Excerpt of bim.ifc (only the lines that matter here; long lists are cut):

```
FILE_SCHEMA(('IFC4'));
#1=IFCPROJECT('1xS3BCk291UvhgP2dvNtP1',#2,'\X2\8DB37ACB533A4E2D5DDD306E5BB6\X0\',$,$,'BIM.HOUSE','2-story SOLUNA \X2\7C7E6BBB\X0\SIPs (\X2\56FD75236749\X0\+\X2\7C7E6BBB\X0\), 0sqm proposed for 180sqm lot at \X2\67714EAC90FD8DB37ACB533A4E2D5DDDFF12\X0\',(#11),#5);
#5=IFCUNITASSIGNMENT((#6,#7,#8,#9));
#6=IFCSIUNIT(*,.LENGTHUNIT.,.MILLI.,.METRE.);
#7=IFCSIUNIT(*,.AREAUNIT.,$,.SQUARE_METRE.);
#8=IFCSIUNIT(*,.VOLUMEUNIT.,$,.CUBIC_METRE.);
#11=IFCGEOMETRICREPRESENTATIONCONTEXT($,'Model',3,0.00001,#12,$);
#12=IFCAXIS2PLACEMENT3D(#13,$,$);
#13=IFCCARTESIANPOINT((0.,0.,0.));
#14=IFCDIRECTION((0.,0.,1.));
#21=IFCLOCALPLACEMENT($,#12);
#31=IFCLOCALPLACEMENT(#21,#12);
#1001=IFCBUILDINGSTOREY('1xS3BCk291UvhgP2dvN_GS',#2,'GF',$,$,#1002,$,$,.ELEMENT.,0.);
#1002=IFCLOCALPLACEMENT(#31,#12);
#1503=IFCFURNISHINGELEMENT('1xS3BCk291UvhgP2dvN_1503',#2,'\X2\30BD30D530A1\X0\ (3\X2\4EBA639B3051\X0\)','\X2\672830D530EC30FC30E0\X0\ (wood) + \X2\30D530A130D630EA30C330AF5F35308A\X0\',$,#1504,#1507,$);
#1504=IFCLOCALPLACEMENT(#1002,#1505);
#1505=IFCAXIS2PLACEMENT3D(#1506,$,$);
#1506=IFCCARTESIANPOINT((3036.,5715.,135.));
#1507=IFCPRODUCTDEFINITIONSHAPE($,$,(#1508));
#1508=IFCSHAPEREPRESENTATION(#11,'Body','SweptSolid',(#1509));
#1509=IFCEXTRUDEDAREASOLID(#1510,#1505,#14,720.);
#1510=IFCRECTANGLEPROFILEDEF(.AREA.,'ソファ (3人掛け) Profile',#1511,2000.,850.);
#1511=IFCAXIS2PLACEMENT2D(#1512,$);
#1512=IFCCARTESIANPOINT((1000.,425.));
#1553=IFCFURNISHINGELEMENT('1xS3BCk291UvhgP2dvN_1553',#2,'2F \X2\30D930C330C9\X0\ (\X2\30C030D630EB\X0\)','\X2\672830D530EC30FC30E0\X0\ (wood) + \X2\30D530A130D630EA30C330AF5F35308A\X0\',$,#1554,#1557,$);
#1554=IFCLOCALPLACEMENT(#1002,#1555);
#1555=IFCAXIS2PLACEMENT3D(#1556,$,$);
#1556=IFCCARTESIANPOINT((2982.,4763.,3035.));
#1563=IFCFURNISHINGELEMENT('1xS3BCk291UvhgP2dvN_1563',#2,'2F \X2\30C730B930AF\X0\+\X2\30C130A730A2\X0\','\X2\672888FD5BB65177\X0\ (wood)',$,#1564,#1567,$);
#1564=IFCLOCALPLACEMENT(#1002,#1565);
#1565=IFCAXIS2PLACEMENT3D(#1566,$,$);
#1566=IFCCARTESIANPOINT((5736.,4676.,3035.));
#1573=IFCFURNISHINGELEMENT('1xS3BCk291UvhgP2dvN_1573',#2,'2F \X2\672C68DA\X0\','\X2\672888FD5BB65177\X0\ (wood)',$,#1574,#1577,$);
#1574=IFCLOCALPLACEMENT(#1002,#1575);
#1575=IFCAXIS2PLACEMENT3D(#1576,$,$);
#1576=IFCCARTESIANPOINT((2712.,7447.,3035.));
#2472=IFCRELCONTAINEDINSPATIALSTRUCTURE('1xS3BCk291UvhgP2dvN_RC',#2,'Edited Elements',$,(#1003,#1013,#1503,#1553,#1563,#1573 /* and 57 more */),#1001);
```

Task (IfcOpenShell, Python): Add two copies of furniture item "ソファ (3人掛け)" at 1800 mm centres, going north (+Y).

```python
import numpy as np
import ifcopenshell
import ifcopenshell.api.geometry
import ifcopenshell.api.root
import ifcopenshell.util.element
import ifcopenshell.util.placement
import ifcopenshell.util.unit

model = ifcopenshell.open("bim.ifc")
unit_scale = ifcopenshell.util.unit.calculate_unit_scale(model)


def reuse_history(source, copy):
    """copy_class also copies each property set's owner history, people and application; keep the originals."""
    for rel in copy.IsDefinedBy:
        if rel.is_a("IfcRelDefinesByProperties") and (history := rel.RelatingPropertyDefinition.OwnerHistory):
            rel.RelatingPropertyDefinition.OwnerHistory = source.OwnerHistory
            ifcopenshell.util.element.remove_deep2(model, history)


source = model.by_guid("1xS3BCk291UvhgP2dvN_1503")
base = ifcopenshell.util.placement.get_local_placement(source.ObjectPlacement)
step = np.array([0.0, 1.0, 0.0]) * 1.8 / unit_scale

for i in range(1, 3):
    copy = ifcopenshell.api.root.copy_class(model, product=source)
    copy.Representation = ifcopenshell.util.element.copy_deep(
        model, source.Representation, exclude=["IfcGeometricRepresentationContext", "IfcRepresentationMap"]
    )
    reuse_history(source, copy)
    matrix = base.copy()
    matrix[:3, 3] += i * step
    print("added at", matrix[:3, 3].round(3) + 0.0)
    ifcopenshell.api.geometry.edit_object_placement(model, product=copy, matrix=matrix, is_si=False)

model.write("bim-out.ifc")
```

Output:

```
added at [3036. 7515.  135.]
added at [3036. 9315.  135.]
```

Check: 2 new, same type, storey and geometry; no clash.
